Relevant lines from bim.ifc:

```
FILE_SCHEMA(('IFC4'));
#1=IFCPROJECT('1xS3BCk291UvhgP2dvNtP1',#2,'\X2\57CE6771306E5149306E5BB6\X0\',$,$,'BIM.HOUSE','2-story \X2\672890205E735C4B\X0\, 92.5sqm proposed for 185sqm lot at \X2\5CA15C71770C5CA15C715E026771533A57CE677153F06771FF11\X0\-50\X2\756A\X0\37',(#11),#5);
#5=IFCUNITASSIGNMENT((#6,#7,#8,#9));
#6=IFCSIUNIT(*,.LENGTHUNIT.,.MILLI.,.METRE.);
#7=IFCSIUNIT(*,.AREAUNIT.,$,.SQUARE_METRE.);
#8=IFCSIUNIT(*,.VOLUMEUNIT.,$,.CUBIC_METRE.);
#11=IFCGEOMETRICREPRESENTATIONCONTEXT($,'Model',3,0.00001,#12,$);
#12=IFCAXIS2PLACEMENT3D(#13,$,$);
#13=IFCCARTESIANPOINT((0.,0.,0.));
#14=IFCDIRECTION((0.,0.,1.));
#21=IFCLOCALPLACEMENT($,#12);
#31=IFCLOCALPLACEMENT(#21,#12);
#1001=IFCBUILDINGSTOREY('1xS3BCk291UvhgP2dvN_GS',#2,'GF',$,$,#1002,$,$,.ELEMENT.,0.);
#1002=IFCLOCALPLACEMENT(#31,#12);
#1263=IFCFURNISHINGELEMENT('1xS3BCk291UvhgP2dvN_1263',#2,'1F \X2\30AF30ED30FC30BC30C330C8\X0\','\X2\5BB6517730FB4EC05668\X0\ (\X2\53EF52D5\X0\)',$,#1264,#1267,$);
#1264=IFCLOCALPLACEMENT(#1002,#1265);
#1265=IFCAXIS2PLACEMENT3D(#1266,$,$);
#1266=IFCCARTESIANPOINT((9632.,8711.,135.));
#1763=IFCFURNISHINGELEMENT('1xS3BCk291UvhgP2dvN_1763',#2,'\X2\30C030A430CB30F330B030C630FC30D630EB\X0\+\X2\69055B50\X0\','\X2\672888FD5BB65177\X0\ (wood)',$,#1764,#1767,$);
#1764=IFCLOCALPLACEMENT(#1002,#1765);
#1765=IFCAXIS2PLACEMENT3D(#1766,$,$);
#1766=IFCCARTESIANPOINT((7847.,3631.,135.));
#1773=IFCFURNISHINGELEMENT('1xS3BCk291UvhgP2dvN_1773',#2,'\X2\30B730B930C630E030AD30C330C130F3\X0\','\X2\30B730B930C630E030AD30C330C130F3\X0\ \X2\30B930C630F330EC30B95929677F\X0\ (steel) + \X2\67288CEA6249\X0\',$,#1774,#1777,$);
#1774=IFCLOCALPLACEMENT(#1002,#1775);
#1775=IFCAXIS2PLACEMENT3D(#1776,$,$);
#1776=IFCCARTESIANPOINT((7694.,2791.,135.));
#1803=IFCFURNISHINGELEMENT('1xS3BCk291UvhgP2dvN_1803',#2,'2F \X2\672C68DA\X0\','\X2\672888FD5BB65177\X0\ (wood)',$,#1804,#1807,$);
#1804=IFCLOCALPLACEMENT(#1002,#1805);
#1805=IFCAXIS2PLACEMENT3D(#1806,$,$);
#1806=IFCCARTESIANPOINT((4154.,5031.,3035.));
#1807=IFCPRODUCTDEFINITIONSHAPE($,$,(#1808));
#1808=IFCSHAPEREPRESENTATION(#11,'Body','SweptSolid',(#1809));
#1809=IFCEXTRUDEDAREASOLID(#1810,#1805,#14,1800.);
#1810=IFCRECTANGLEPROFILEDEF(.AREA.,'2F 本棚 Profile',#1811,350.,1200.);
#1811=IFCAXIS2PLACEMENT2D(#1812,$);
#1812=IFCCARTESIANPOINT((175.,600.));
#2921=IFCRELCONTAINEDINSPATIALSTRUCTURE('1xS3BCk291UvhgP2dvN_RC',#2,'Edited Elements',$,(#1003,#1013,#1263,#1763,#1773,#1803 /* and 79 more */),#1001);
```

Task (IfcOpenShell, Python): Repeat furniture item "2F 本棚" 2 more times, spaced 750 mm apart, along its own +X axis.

```python
import ifcopenshell
import ifcopenshell.api.geometry
import ifcopenshell.api.root
import ifcopenshell.util.element
import ifcopenshell.util.placement

model = ifcopenshell.open("bim.ifc")


def reuse_history(source, copy):
    """copy_class also copies each property set's owner history, people and application; keep the originals."""
    for rel in copy.IsDefinedBy:
        if rel.is_a("IfcRelDefinesByProperties") and (history := rel.RelatingPropertyDefinition.OwnerHistory):
            rel.RelatingPropertyDefinition.OwnerHistory = source.OwnerHistory
            ifcopenshell.util.element.remove_deep2(model, history)


source = model.by_guid("1xS3BCk291UvhgP2dvN_1803")
base = ifcopenshell.util.placement.get_local_placement(source.ObjectPlacement)
step = base[:3, 0] * 750.0

for i in range(1, 3):
    copy = ifcopenshell.api.root.copy_class(model, product=source)
    copy.Representation = ifcopenshell.util.element.copy_deep(
        model, source.Representation, exclude=["IfcGeometricRepresentationContext", "IfcRepresentationMap"]
    )
    reuse_history(source, copy)
    matrix = base.copy()
    matrix[:3, 3] += i * step
    print("added at", matrix[:3, 3].round(3) + 0.0)
    ifcopenshell.api.geometry.edit_object_placement(model, product=copy, matrix=matrix, is_si=False)

model.write("bim_edited.ifc")
```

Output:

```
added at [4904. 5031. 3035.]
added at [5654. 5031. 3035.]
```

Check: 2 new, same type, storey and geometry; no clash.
